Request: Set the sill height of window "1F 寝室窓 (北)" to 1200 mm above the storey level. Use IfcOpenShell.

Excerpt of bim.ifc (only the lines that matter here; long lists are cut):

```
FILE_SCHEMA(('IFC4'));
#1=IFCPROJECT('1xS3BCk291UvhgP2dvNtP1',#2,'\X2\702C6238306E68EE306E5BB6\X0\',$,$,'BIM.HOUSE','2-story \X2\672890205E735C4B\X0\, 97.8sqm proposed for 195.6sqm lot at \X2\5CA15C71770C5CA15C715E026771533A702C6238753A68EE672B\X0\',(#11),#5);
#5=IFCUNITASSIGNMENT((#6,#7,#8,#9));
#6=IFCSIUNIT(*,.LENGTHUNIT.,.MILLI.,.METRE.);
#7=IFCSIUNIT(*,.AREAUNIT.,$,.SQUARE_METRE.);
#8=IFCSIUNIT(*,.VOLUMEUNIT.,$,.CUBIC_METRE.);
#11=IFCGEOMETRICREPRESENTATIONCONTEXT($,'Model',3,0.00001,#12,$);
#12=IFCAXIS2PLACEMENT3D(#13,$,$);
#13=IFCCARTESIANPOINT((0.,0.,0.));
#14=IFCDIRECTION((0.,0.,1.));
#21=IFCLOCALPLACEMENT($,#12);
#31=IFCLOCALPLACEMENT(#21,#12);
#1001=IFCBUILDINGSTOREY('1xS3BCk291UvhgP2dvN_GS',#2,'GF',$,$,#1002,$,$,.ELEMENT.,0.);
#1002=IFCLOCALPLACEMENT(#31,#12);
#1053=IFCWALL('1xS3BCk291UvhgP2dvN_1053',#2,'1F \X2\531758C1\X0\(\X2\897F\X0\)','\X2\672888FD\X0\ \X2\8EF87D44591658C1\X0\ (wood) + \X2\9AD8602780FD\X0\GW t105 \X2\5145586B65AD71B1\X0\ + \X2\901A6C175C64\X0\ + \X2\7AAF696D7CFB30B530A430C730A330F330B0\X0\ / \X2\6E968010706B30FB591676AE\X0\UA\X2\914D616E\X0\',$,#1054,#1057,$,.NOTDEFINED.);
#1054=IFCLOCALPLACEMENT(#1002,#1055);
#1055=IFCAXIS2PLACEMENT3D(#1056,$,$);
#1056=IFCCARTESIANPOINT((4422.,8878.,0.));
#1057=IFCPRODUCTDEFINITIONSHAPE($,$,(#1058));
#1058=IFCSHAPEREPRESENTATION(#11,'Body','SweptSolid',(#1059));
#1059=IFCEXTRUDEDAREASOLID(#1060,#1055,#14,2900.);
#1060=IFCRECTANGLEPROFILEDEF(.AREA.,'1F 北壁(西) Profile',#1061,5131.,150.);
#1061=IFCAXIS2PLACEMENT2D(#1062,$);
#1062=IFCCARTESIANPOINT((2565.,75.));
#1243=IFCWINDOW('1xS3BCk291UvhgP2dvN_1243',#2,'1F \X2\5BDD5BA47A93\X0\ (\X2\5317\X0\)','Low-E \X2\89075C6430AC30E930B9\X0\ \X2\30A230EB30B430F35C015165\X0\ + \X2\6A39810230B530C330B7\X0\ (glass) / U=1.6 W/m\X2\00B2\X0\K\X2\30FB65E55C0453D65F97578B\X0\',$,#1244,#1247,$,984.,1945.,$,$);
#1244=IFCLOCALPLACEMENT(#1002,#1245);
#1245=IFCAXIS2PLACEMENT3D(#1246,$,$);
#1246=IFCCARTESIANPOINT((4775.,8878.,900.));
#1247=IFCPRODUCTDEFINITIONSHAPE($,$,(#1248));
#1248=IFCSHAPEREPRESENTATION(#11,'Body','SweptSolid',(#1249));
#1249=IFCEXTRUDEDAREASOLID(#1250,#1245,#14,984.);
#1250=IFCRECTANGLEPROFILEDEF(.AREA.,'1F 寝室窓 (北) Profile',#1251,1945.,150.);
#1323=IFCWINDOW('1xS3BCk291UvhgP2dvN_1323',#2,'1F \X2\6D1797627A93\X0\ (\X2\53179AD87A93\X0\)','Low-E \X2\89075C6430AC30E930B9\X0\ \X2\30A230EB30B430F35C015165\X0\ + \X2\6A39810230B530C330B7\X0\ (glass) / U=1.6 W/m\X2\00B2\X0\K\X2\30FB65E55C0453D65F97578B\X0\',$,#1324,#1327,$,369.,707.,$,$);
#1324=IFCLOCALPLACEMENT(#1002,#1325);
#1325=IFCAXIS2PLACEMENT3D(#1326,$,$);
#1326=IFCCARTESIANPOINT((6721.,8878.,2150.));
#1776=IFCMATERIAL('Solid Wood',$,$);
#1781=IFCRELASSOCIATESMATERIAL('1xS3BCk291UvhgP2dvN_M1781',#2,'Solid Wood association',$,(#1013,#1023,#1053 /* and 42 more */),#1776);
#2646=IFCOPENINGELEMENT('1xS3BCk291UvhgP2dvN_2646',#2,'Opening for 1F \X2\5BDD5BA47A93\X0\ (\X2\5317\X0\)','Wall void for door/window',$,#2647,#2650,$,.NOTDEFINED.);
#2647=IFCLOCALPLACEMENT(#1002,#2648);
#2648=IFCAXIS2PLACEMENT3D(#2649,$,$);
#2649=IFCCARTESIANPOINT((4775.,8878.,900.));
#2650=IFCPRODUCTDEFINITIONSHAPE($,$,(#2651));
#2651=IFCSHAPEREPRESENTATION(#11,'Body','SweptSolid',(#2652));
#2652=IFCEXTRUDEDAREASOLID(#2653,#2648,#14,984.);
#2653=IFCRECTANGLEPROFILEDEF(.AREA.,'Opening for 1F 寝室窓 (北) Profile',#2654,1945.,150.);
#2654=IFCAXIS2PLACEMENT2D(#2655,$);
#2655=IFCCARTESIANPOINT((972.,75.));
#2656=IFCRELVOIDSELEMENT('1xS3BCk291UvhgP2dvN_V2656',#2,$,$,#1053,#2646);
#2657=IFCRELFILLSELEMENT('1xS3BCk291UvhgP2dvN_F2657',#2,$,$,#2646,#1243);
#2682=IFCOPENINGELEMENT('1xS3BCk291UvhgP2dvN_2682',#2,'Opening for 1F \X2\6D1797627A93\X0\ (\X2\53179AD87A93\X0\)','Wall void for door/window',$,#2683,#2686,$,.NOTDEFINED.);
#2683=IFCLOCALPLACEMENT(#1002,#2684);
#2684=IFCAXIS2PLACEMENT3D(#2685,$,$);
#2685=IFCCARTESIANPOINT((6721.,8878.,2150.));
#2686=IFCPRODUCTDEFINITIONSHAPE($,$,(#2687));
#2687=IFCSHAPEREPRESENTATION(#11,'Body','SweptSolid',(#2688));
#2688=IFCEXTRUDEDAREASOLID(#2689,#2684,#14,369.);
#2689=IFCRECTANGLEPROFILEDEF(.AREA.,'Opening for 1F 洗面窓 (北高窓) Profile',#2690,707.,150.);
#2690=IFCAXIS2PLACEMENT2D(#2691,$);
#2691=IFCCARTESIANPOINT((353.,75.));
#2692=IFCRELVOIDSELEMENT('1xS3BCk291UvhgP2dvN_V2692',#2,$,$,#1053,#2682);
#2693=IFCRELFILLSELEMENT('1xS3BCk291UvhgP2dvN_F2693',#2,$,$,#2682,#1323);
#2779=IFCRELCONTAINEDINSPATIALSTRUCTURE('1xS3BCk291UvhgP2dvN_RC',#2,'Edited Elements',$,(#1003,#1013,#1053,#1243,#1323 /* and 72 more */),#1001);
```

```python
import numpy as np
import ifcopenshell
import ifcopenshell.api.geometry
import ifcopenshell.geom
import ifcopenshell.util.element
import ifcopenshell.util.placement
import ifcopenshell.util.shape
import ifcopenshell.util.unit

model = ifcopenshell.open("bim.ifc")
unit_scale = ifcopenshell.util.unit.calculate_unit_scale(model)

window = model.by_guid("1xS3BCk291UvhgP2dvN_1243")
opening = window.FillsVoids[0].RelatingOpeningElement
storey = ifcopenshell.util.element.get_container(window, ifc_class="IfcBuildingStorey")
level = ifcopenshell.util.placement.get_local_placement(storey.ObjectPlacement)[2, 3]

# The opening's origin need not be at the sill, so measure its lowest point.
shape = ifcopenshell.geom.create_shape(ifcopenshell.geom.settings(), opening)
bottom = ifcopenshell.util.shape.get_shape_bottom_elevation(shape, shape.geometry) / unit_scale
dz = level + 1200.0 - bottom

shift = np.array([0.0, 0.0, dz])
# The window is not placed relative to its opening, so move both.
for product in (opening, window):
    matrix = ifcopenshell.util.placement.get_local_placement(product.ObjectPlacement)
    matrix[:3, 3] += shift
    ifcopenshell.api.geometry.edit_object_placement(model, product=product, matrix=matrix, is_si=False)

print(f"moved by {dz * unit_scale:+.3f} m")

model.write("bim_edited.ifc")
```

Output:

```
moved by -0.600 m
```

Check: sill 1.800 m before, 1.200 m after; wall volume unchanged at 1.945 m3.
